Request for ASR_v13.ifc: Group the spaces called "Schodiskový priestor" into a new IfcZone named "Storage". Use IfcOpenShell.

First a look at what the model holds.

```python
import ifcopenshell

model = ifcopenshell.open("ASR_v13.ifc")
print(model.schema)
seen = {}
for space in model.by_type("IfcSpace"):
    seen[space.LongName] = seen.get(space.LongName, 0) + 1
for name, count in sorted(seen.items(), key=str):
    print(count, "x", name)
print("zones:", [z.Name for z in model.by_type("IfcZone")][:20])
```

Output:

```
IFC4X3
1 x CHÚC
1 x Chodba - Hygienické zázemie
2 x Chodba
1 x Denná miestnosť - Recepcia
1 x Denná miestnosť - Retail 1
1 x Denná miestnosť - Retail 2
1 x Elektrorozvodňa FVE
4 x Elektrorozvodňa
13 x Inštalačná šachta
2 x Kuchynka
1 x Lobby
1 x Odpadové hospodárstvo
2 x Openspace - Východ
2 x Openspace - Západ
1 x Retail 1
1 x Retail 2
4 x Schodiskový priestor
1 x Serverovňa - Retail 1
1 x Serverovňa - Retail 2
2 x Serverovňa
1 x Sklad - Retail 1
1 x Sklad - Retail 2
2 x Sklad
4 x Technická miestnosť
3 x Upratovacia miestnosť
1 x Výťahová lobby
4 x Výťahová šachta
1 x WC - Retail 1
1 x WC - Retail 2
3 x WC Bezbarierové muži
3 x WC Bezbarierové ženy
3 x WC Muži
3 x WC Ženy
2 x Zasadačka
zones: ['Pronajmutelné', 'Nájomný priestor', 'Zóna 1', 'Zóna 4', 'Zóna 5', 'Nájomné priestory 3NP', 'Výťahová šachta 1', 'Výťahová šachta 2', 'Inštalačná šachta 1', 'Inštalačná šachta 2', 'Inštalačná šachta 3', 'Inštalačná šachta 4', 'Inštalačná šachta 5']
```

```python
import ifcopenshell
import ifcopenshell.api.group
import ifcopenshell.api.root

model = ifcopenshell.open("ASR_v13.ifc")

names = {"Schodiskový priestor"}
spaces = [s for s in model.by_type("IfcSpace") if s.LongName in names]

zone = ifcopenshell.api.root.create_entity(model, ifc_class="IfcZone", name="Storage")
ifcopenshell.api.group.assign_group(model, products=spaces, group=zone)
print(len(spaces), "spaces in", zone.Name)

model.write("ASR_v13_v2.ifc")
```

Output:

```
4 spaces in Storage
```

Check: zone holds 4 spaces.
